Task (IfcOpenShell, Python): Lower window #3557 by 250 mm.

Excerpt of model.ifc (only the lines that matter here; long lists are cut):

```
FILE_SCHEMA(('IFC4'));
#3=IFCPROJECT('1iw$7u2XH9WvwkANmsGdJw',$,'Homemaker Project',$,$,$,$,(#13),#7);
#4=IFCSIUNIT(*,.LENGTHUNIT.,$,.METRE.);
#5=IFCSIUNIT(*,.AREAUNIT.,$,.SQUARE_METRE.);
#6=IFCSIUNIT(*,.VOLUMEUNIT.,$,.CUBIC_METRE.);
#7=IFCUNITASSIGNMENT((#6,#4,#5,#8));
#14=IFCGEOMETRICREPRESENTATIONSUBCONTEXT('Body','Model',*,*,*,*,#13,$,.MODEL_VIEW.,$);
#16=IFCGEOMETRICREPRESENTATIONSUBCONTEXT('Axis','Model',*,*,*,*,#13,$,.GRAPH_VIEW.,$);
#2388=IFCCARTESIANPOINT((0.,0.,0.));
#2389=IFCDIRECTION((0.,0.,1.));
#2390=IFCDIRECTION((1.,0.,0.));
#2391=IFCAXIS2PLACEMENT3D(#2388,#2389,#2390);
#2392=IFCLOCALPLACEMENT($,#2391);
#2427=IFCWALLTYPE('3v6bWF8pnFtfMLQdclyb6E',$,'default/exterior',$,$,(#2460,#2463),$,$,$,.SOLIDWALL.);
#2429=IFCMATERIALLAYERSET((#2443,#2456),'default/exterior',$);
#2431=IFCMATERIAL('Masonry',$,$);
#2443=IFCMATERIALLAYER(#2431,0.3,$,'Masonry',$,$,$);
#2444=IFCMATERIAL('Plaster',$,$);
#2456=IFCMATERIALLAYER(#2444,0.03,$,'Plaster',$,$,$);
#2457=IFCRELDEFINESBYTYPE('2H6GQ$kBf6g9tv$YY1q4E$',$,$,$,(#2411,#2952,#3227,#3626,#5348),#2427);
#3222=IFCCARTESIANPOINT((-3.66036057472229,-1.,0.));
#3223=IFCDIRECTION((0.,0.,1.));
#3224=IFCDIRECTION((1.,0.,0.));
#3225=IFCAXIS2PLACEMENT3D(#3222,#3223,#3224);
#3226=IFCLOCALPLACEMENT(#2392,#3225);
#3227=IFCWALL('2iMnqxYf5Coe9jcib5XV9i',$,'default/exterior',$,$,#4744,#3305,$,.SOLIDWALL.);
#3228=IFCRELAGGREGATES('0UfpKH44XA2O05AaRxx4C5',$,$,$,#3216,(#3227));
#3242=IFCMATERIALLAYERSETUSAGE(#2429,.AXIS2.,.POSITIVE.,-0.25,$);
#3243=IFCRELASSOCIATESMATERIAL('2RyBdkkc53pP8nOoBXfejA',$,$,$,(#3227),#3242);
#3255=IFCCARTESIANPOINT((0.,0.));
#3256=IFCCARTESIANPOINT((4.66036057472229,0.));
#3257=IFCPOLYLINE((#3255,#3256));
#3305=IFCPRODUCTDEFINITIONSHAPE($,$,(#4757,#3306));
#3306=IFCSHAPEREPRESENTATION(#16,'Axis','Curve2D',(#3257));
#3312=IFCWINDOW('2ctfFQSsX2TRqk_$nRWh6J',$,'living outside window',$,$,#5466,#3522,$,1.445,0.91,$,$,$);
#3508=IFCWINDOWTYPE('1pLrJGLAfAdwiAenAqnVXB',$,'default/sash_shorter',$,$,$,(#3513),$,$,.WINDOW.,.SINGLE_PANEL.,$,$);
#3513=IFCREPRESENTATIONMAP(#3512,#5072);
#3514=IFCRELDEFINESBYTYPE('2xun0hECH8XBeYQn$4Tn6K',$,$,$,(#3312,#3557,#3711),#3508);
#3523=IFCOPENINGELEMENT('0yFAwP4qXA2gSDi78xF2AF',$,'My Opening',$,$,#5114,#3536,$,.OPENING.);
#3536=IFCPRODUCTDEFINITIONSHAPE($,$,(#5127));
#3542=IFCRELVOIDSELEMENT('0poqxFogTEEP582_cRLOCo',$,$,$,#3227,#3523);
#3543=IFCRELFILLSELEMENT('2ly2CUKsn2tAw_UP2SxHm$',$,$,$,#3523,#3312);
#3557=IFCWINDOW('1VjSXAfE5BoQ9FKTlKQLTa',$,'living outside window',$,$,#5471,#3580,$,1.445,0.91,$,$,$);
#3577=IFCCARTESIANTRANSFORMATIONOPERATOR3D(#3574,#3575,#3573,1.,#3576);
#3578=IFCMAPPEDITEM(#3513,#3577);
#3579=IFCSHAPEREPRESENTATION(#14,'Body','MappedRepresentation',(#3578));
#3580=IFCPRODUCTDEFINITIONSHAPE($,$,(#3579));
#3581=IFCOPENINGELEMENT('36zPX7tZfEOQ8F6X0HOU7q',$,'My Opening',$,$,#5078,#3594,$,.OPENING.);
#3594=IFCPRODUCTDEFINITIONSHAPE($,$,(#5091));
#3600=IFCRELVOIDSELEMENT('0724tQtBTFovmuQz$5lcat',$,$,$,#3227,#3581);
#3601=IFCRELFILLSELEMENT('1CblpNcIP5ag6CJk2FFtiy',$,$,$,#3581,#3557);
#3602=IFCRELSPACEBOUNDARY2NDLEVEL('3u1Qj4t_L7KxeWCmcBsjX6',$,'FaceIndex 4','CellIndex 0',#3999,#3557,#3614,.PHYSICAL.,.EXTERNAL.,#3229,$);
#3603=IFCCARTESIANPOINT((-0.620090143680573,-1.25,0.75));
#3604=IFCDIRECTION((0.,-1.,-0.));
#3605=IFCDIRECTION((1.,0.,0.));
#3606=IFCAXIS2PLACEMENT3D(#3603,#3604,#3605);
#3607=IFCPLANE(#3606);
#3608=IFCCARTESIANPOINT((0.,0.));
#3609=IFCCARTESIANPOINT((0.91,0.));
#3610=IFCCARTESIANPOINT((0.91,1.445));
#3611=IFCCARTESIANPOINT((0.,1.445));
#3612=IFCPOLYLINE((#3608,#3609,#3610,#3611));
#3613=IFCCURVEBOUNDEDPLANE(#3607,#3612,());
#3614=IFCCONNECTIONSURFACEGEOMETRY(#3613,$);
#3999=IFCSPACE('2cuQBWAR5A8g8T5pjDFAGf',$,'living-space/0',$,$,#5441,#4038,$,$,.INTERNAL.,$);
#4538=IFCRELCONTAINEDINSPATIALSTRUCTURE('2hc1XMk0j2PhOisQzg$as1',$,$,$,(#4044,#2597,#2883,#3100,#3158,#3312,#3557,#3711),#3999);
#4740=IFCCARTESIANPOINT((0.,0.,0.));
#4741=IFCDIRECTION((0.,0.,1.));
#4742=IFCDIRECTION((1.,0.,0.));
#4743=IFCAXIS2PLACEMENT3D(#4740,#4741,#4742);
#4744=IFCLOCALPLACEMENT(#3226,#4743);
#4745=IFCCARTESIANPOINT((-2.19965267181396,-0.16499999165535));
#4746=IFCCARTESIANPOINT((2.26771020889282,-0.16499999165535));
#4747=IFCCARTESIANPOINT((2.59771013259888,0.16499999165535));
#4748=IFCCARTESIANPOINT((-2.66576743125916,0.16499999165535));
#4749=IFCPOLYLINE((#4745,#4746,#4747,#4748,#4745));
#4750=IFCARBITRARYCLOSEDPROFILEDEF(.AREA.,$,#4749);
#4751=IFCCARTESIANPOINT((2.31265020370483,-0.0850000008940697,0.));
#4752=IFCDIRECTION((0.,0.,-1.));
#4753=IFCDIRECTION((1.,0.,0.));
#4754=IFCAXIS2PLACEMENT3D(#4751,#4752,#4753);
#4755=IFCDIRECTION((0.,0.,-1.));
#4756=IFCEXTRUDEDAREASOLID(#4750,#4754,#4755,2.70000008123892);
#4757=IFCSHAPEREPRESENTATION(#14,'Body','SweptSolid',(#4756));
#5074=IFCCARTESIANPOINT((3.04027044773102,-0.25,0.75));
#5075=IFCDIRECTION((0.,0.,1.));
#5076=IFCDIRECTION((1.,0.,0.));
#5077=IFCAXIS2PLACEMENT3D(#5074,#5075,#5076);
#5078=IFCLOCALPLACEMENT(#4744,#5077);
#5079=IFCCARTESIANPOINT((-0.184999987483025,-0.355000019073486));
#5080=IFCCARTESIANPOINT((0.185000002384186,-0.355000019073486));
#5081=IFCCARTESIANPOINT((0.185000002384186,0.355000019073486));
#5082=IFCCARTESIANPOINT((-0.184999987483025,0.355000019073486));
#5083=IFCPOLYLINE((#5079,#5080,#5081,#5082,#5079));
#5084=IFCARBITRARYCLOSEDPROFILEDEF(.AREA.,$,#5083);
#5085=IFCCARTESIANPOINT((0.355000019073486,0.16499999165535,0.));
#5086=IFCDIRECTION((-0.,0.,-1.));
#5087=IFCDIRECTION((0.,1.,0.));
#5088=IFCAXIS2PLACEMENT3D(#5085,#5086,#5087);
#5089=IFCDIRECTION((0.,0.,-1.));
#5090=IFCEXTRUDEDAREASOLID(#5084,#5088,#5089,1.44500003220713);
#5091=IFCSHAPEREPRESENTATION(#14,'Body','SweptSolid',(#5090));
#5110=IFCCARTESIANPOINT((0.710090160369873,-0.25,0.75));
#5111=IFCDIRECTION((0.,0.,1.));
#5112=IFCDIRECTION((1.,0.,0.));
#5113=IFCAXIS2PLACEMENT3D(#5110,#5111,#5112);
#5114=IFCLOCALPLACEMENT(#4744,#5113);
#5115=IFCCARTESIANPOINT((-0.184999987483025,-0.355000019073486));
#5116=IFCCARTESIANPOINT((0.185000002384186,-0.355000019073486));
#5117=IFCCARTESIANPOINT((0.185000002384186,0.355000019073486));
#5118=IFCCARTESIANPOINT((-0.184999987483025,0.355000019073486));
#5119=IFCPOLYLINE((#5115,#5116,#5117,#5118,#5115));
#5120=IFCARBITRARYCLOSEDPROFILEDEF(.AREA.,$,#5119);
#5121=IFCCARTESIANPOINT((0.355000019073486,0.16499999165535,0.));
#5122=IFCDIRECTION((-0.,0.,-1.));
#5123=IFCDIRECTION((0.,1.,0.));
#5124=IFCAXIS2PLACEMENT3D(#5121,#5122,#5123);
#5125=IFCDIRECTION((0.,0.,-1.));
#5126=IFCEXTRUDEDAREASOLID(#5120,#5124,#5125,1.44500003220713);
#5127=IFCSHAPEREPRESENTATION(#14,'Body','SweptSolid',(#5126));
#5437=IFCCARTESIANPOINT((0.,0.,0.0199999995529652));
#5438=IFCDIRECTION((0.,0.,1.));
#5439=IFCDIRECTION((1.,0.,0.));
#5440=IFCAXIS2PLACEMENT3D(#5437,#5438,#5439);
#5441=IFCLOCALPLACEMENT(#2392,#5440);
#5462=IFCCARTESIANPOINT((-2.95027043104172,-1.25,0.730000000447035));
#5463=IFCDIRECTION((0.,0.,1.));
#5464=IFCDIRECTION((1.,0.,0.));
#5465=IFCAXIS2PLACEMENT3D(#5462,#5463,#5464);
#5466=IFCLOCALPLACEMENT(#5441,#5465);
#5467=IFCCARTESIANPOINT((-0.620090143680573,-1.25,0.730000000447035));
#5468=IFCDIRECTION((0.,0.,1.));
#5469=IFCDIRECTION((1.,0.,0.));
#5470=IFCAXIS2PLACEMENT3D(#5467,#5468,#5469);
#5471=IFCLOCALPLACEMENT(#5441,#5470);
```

```python
import numpy as np
import ifcopenshell
import ifcopenshell.api.geometry
import ifcopenshell.util.placement
import ifcopenshell.util.unit

model = ifcopenshell.open("model.ifc")
unit_scale = ifcopenshell.util.unit.calculate_unit_scale(model)

window = model.by_guid("1VjSXAfE5BoQ9FKTlKQLTa")
opening = window.FillsVoids[0].RelatingOpeningElement
dz = -0.25 / unit_scale

shift = np.array([0.0, 0.0, dz])
# The window is not placed relative to its opening, so move both.
for product in (opening, window):
    matrix = ifcopenshell.util.placement.get_local_placement(product.ObjectPlacement)
    matrix[:3, 3] += shift
    ifcopenshell.api.geometry.edit_object_placement(model, product=product, matrix=matrix, is_si=False)

# Space boundary surfaces are stored in each space's coordinates; move them too.
for rel in window.ProvidesBoundaries:
    if not rel.ConnectionGeometry:
        continue
    surface = rel.ConnectionGeometry.SurfaceOnRelatingElement.BasisSurface
    space_matrix = ifcopenshell.util.placement.get_local_placement(rel.RelatingSpace.ObjectPlacement)
    point = np.array(surface.Position.Location.Coordinates) + space_matrix[:3, :3].T @ shift
    surface.Position = model.createIfcAxis2Placement3D(
        model.createIfcCartesianPoint(point.tolist()), surface.Position.Axis, surface.Position.RefDirection
    )

print(f"moved by {dz * unit_scale:+.3f} m")

model.write("model-out.ifc")
```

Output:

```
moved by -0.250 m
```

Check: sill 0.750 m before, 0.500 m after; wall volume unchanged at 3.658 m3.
